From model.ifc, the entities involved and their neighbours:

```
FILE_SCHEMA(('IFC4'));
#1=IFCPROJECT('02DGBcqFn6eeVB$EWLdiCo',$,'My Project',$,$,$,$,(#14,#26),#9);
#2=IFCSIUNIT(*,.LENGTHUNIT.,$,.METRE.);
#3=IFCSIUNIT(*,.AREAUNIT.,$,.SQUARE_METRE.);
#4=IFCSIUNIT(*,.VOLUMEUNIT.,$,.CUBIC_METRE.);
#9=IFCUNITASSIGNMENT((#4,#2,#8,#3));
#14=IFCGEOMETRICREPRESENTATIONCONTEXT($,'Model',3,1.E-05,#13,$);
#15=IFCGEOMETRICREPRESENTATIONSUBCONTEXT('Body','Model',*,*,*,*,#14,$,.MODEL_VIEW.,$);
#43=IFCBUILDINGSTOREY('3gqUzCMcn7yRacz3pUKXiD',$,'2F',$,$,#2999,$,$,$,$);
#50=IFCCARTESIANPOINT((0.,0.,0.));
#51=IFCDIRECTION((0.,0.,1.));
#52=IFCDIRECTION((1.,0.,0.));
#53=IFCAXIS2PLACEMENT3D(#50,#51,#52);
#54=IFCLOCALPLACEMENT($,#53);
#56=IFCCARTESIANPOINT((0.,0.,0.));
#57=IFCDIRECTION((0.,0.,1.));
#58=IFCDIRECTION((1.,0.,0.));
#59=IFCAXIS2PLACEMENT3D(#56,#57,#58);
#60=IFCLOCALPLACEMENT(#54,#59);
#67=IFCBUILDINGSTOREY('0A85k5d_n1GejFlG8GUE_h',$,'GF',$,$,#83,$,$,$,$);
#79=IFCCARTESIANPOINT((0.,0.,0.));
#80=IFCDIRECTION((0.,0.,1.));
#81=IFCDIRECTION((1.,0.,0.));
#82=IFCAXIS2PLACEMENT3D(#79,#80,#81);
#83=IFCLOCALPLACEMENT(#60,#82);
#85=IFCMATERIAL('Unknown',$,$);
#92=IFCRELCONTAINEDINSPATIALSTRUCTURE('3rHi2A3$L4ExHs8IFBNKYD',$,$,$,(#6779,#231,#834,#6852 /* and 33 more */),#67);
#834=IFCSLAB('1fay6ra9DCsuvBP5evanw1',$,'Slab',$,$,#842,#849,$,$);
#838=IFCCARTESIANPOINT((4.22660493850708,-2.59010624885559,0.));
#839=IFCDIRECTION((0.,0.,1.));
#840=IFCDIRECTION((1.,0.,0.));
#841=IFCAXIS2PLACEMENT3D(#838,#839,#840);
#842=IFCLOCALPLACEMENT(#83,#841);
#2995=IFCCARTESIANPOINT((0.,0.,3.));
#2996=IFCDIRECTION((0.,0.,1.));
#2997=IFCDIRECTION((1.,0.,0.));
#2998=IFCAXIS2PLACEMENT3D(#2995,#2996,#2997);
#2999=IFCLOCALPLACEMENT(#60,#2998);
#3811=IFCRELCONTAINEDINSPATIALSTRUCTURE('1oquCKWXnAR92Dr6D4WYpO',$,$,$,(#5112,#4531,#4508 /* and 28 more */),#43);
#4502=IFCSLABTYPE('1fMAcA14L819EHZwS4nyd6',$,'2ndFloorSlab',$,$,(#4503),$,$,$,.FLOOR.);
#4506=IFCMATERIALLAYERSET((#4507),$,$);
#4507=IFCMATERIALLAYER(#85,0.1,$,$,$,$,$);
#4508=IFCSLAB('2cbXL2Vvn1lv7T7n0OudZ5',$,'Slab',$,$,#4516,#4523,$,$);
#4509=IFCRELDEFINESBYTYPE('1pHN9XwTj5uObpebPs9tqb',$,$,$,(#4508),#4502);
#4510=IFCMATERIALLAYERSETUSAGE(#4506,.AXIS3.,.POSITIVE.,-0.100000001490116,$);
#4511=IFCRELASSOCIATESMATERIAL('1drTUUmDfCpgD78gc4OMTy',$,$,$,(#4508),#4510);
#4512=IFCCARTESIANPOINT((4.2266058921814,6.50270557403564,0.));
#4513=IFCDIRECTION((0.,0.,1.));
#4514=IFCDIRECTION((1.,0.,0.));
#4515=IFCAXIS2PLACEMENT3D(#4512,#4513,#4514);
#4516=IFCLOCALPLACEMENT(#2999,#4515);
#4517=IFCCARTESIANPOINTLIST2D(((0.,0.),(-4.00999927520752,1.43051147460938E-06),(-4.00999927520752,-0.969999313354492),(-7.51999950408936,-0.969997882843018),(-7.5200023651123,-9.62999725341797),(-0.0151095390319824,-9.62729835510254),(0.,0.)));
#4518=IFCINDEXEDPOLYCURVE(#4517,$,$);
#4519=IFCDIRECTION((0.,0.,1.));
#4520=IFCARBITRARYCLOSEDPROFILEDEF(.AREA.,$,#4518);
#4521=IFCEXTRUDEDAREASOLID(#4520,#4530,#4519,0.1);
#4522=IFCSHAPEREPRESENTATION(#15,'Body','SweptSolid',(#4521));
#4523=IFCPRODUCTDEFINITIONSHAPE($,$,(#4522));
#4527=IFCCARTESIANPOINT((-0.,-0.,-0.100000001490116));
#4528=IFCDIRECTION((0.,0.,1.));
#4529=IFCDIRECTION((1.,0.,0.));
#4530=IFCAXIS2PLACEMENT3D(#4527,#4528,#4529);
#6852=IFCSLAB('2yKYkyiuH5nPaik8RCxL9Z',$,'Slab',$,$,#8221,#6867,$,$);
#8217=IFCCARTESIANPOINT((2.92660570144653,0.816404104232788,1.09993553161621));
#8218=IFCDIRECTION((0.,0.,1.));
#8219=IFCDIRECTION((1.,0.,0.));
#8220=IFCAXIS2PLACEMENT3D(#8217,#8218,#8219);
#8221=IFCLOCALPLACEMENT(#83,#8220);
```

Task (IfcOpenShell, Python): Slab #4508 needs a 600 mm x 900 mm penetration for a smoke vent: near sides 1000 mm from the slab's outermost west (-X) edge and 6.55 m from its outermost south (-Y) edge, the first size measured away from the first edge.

```python
import numpy as np
import ifcopenshell
import ifcopenshell.api.feature
import ifcopenshell.api.geometry
import ifcopenshell.api.root
import ifcopenshell.geom
import ifcopenshell.util.placement
import ifcopenshell.util.representation
import ifcopenshell.util.shape
import ifcopenshell.util.unit

model = ifcopenshell.open("model.ifc")
unit_scale = ifcopenshell.util.unit.calculate_unit_scale(model)
settings = ifcopenshell.geom.settings()


def volume(element):
    """Net volume in cubic metres, openings subtracted."""
    shape = ifcopenshell.geom.create_shape(settings, element)
    return ifcopenshell.util.shape.get_volume(shape.geometry)


slab = model.by_guid("2cbXL2Vvn1lv7T7n0OudZ5")
before = volume(slab)

# Extent in the slab's own axes, in metres. The edges named are its -X and -Y sides.
slab_shape = ifcopenshell.geom.create_shape(settings, slab)
vertices = ifcopenshell.util.shape.get_vertices(slab_shape.geometry)
x_min, y_min, bottom = vertices.min(axis=0)
top = vertices[:, 2].max()

opening = ifcopenshell.api.root.create_entity(model, ifc_class="IfcOpeningElement", name="Smoke vent opening", predefined_type="OPENING")
context = ifcopenshell.util.representation.get_context(model, "Model", "Body", "MODEL_VIEW")
width, depth = 0.6, 0.9
outline = [(0.0, 0.0), (width, 0.0), (width, depth), (0.0, depth), (0.0, 0.0)]
# Overshoot both faces by 50 mm so the cut is clean.
shape = ifcopenshell.api.geometry.add_slab_representation(
    model, context=context, depth=top - bottom + 0.1, polyline=outline
)
ifcopenshell.api.geometry.assign_representation(model, product=opening, representation=shape)

matrix = ifcopenshell.util.placement.get_local_placement(slab.ObjectPlacement)
matrix[:, 3] = matrix @ np.append(np.array([x_min + 1, y_min + 6.55, bottom - 0.05]) / unit_scale, 1.0)
ifcopenshell.api.geometry.edit_object_placement(model, product=opening, matrix=matrix, is_si=False)
ifcopenshell.api.feature.add_feature(model, feature=opening, element=slab)

after = volume(slab)

print(f"slab volume {before:.3f} -> {after:.3f} m3")

model.write("model_edited.ifc")
```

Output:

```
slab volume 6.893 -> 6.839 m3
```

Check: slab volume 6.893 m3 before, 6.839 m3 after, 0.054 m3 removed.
